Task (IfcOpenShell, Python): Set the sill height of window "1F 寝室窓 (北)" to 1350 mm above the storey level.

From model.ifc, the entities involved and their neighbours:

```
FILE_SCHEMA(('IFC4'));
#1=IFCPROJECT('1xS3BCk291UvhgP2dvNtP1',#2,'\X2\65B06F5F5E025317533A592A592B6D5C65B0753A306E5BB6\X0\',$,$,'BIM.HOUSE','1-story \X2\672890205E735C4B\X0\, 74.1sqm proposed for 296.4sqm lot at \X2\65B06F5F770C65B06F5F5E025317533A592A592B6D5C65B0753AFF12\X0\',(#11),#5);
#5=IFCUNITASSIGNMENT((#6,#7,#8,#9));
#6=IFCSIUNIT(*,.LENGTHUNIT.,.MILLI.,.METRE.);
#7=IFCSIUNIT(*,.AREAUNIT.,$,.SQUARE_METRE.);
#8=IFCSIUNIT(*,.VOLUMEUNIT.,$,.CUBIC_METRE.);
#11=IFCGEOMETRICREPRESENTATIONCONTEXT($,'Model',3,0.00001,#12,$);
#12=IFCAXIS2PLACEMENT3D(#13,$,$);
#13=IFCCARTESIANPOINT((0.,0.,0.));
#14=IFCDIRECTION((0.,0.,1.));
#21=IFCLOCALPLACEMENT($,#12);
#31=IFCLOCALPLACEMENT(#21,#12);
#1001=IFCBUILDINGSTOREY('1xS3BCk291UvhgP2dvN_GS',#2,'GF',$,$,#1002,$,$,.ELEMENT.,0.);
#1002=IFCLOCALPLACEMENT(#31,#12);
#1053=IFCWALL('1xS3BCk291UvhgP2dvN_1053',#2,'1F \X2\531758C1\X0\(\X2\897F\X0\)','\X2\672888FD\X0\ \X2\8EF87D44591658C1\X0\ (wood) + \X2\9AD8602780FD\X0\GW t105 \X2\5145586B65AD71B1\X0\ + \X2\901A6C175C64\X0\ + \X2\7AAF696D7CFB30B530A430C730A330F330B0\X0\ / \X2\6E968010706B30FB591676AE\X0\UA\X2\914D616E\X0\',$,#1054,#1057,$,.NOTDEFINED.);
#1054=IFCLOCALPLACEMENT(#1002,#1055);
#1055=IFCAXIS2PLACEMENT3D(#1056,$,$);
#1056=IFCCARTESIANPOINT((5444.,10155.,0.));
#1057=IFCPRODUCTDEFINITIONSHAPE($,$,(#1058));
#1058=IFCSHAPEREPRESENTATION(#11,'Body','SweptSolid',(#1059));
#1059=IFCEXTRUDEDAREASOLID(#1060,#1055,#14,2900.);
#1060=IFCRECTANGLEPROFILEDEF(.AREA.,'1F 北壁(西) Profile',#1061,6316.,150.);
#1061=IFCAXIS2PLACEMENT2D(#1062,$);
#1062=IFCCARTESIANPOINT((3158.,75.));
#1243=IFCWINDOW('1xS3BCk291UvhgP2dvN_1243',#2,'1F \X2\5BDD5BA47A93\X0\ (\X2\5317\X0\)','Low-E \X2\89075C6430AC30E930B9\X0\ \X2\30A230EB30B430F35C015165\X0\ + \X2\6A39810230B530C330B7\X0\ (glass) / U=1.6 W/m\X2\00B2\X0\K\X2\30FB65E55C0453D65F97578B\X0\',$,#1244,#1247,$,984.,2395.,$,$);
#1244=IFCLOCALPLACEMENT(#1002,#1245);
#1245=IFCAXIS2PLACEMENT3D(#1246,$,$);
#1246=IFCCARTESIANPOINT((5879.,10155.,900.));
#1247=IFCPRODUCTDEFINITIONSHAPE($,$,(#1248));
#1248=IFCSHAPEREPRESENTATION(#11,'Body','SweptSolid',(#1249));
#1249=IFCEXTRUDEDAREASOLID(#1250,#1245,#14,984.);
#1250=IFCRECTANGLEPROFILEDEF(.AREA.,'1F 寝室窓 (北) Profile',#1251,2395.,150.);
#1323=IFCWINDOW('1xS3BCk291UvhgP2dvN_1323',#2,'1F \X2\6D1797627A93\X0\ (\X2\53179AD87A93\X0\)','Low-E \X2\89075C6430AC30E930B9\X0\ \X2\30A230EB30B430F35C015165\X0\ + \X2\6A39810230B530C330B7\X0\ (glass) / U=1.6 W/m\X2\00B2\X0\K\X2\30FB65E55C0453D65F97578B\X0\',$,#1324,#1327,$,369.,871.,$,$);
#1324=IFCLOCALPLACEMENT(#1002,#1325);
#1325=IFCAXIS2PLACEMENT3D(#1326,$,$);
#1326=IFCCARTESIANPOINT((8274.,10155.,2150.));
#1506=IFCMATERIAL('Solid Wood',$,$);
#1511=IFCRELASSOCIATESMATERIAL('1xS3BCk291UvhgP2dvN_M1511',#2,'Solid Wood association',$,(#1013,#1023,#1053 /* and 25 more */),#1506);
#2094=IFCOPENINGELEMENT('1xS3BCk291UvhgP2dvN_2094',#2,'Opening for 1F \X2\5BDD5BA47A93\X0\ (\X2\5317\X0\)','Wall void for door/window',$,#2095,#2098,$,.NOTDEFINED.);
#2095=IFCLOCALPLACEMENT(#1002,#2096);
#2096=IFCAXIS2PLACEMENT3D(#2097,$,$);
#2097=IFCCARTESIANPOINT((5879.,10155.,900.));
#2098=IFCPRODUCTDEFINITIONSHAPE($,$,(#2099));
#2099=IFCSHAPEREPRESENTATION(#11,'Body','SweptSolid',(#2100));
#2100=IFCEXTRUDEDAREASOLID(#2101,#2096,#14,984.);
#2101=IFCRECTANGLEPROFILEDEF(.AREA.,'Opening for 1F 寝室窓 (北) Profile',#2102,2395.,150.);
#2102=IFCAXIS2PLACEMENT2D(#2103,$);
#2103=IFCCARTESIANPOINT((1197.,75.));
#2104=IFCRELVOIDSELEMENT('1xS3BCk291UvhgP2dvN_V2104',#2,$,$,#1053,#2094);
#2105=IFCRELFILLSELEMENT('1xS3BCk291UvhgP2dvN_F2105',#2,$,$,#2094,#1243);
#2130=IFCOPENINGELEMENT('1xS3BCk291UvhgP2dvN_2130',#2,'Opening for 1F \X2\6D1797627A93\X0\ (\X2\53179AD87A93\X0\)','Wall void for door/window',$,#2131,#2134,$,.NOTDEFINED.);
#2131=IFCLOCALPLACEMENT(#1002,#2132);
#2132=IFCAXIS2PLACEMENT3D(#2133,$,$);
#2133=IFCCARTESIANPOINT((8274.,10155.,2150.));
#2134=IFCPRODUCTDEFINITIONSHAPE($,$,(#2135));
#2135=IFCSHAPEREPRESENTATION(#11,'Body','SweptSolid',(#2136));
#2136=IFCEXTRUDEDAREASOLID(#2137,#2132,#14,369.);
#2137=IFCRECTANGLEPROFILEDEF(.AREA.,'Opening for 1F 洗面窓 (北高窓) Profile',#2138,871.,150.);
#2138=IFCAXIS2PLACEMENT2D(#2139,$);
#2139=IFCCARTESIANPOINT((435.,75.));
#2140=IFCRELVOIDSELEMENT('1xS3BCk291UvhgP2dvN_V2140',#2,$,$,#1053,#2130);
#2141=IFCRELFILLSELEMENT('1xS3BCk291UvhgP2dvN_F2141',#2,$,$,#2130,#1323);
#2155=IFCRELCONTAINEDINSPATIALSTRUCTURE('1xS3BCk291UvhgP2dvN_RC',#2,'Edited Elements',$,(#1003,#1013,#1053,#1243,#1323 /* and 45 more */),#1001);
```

```python
import numpy as np
import ifcopenshell
import ifcopenshell.api.geometry
import ifcopenshell.geom
import ifcopenshell.util.element
import ifcopenshell.util.placement
import ifcopenshell.util.shape
import ifcopenshell.util.unit

model = ifcopenshell.open("model.ifc")
unit_scale = ifcopenshell.util.unit.calculate_unit_scale(model)

window = model.by_guid("1xS3BCk291UvhgP2dvN_1243")
opening = window.FillsVoids[0].RelatingOpeningElement
storey = ifcopenshell.util.element.get_container(window, ifc_class="IfcBuildingStorey")
level = ifcopenshell.util.placement.get_local_placement(storey.ObjectPlacement)[2, 3]

# The opening's origin need not be at the sill, so measure its lowest point.
shape = ifcopenshell.geom.create_shape(ifcopenshell.geom.settings(), opening)
bottom = ifcopenshell.util.shape.get_shape_bottom_elevation(shape, shape.geometry) / unit_scale
dz = level + 1.35 / unit_scale - bottom

shift = np.array([0.0, 0.0, dz])
# The window is not placed relative to its opening, so move both.
for product in (opening, window):
    matrix = ifcopenshell.util.placement.get_local_placement(product.ObjectPlacement)
    matrix[:3, 3] += shift
    ifcopenshell.api.geometry.edit_object_placement(model, product=product, matrix=matrix, is_si=False)

print(f"moved by {dz * unit_scale:+.3f} m")

model.write("model_rev.ifc")
```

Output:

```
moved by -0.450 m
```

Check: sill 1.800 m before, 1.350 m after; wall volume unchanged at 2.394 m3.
